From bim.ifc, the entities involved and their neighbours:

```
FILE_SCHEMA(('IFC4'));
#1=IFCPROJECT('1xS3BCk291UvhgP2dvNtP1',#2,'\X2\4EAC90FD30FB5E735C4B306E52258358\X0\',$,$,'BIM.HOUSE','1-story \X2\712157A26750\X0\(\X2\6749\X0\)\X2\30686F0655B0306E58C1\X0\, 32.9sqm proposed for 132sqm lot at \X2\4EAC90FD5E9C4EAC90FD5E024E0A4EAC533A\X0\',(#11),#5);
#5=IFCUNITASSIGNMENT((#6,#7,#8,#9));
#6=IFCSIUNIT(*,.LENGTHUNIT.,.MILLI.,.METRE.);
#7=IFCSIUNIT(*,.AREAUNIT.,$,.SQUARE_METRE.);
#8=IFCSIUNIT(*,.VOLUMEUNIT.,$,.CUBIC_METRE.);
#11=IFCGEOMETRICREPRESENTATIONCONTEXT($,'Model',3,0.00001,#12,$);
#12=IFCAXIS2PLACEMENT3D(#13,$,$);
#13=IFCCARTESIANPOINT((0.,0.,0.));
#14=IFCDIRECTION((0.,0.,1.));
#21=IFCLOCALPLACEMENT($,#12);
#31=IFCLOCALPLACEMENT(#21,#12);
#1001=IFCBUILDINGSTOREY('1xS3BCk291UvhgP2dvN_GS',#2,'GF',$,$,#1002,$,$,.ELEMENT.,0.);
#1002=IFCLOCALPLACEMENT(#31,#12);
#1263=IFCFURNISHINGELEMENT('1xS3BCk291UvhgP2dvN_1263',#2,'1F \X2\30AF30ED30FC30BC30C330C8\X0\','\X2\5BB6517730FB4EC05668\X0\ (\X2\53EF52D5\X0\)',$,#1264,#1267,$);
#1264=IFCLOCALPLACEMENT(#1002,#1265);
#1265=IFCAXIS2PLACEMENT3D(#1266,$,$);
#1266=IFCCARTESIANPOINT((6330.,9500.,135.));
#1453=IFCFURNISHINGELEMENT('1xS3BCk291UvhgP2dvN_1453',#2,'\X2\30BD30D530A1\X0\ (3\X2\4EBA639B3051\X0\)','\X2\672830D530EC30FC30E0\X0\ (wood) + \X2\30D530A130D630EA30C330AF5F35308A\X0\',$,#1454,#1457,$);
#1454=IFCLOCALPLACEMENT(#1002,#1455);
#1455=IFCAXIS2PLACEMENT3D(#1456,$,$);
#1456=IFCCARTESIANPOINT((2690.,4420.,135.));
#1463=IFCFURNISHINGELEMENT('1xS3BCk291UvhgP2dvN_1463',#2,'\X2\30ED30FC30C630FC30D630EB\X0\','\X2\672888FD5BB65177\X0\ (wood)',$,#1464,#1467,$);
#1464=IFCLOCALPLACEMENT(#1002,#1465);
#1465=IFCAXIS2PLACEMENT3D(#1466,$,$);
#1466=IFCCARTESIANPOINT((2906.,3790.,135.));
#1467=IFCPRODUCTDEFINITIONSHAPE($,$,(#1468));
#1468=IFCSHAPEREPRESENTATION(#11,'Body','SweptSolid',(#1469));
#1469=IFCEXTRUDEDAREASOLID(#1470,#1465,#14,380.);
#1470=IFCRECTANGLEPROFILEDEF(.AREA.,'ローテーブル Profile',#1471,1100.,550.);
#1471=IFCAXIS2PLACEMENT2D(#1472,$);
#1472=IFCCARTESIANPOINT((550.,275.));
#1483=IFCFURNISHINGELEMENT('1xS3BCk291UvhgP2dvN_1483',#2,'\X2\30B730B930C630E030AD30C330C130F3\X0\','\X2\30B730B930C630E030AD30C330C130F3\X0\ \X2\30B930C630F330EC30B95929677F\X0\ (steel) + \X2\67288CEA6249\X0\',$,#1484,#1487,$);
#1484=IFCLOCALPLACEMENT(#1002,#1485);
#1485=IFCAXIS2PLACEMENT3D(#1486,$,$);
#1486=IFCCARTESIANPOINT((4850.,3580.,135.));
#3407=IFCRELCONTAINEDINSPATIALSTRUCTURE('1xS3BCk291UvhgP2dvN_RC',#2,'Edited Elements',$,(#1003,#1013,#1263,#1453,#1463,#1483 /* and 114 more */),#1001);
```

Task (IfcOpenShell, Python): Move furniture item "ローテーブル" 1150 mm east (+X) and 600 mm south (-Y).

```python
import ifcopenshell
import ifcopenshell.api.geometry
import ifcopenshell.util.placement
import ifcopenshell.util.unit

model = ifcopenshell.open("bim.ifc")
unit_scale = ifcopenshell.util.unit.calculate_unit_scale(model)

item = model.by_guid("1xS3BCk291UvhgP2dvN_1463")
matrix = ifcopenshell.util.placement.get_local_placement(item.ObjectPlacement)
matrix[0, 3] += 1.15 / unit_scale
matrix[1, 3] -= 0.6 / unit_scale
ifcopenshell.api.geometry.edit_object_placement(model, product=item, matrix=matrix, is_si=False)

print(ifcopenshell.util.placement.get_local_placement(item.ObjectPlacement).round(3) + 0.0)

model.write("bim-out.ifc")
```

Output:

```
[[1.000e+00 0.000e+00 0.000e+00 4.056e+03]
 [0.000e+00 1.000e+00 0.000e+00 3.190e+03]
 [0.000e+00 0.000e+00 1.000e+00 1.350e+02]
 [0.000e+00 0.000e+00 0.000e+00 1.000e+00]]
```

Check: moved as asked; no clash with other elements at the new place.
